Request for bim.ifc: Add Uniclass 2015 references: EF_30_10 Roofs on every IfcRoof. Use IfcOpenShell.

First a look at what the model holds.

```python
import ifcopenshell

model = ifcopenshell.open("bim.ifc")
print(model.schema)
print("classifications:", [c.Name for c in model.by_type("IfcClassification")])
for ifc_class in ("IfcDoor", "IfcRoof", "IfcStair", "IfcWall", "IfcWindow"):
    print(ifc_class, len(model.by_type(ifc_class)))
```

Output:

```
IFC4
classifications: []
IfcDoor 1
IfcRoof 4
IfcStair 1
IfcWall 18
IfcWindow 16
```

```python
import ifcopenshell
import ifcopenshell.api.classification

model = ifcopenshell.open("bim.ifc")

system = ifcopenshell.api.classification.add_classification(model, classification="Uniclass 2015")

codes = {
    "IfcRoof": ("EF_30_10", "Roofs"),
}
for ifc_class, (code, name) in codes.items():
    products = model.by_type(ifc_class)
    ifcopenshell.api.classification.add_reference(
        model, products=products, classification=system, identification=code, name=name
    )
    print(code, len(products))

model.write("bim-out.ifc")
```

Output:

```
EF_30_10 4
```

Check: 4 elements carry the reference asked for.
